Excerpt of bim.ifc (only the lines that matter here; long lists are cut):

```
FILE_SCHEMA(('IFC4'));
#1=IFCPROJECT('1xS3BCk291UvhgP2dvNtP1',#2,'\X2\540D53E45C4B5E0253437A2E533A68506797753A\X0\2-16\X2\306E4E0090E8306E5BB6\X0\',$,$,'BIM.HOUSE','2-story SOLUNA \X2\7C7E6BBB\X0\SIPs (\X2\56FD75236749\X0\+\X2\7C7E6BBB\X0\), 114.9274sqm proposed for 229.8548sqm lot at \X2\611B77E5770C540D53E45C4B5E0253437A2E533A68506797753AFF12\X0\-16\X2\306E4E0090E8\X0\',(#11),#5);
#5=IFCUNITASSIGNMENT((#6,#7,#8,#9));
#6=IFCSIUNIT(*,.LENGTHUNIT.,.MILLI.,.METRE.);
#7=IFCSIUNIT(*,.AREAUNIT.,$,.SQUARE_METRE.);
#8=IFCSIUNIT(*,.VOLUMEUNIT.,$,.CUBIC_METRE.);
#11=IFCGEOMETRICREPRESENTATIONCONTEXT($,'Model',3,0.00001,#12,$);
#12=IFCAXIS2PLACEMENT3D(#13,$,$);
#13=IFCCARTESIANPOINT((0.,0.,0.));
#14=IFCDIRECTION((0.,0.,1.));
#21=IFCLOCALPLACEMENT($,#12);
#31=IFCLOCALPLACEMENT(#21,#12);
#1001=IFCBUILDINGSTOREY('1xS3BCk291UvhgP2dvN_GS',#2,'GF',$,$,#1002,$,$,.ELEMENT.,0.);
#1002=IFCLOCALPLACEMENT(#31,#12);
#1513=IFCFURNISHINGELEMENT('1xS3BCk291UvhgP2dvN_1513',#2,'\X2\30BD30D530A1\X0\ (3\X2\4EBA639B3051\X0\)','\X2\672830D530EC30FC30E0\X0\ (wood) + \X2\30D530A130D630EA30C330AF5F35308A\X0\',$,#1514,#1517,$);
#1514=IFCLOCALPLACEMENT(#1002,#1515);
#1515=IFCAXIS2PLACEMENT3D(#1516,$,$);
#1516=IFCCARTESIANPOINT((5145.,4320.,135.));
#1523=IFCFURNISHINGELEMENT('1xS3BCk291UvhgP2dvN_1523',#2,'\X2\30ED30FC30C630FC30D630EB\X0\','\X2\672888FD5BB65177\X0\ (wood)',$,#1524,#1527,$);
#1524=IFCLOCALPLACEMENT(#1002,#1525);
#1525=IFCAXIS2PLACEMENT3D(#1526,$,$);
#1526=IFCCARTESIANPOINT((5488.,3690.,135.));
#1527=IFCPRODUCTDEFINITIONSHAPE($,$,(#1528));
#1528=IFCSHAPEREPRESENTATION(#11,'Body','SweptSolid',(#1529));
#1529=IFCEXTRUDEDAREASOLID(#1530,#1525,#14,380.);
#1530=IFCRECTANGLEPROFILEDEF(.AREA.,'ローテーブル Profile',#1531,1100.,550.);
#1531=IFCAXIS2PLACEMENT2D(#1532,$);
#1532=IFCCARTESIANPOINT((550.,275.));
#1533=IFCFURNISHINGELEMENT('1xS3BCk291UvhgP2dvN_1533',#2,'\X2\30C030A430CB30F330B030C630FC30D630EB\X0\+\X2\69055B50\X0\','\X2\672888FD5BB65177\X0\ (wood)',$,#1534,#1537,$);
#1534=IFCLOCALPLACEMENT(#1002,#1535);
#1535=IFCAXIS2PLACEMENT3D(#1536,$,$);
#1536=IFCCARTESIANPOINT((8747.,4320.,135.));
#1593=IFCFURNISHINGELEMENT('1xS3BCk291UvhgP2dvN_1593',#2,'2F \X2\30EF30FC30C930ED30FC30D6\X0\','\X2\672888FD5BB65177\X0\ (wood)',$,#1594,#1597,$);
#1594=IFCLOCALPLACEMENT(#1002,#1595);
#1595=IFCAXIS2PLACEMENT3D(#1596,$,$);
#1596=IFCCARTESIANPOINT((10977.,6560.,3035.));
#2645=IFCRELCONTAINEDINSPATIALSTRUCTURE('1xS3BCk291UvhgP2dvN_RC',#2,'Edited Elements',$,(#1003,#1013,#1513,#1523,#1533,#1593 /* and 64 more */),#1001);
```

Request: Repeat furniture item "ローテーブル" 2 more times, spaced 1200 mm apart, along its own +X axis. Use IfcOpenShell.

```python
import ifcopenshell
import ifcopenshell.api.geometry
import ifcopenshell.api.root
import ifcopenshell.util.element
import ifcopenshell.util.placement

model = ifcopenshell.open("bim.ifc")


def reuse_history(source, copy):
    """copy_class also copies each property set's owner history, people and application; keep the originals."""
    for rel in copy.IsDefinedBy:
        if rel.is_a("IfcRelDefinesByProperties") and (history := rel.RelatingPropertyDefinition.OwnerHistory):
            rel.RelatingPropertyDefinition.OwnerHistory = source.OwnerHistory
            ifcopenshell.util.element.remove_deep2(model, history)


source = model.by_id(1523)
base = ifcopenshell.util.placement.get_local_placement(source.ObjectPlacement)
step = base[:3, 0] * 1200.0

for i in range(1, 3):
    copy = ifcopenshell.api.root.copy_class(model, product=source)
    copy.Representation = ifcopenshell.util.element.copy_deep(
        model, source.Representation, exclude=["IfcGeometricRepresentationContext", "IfcRepresentationMap"]
    )
    reuse_history(source, copy)
    matrix = base.copy()
    matrix[:3, 3] += i * step
    print("added at", matrix[:3, 3].round(3) + 0.0)
    ifcopenshell.api.geometry.edit_object_placement(model, product=copy, matrix=matrix, is_si=False)

model.write("bim_updated.ifc")
```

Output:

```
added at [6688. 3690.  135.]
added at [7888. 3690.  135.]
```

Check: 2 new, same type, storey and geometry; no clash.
